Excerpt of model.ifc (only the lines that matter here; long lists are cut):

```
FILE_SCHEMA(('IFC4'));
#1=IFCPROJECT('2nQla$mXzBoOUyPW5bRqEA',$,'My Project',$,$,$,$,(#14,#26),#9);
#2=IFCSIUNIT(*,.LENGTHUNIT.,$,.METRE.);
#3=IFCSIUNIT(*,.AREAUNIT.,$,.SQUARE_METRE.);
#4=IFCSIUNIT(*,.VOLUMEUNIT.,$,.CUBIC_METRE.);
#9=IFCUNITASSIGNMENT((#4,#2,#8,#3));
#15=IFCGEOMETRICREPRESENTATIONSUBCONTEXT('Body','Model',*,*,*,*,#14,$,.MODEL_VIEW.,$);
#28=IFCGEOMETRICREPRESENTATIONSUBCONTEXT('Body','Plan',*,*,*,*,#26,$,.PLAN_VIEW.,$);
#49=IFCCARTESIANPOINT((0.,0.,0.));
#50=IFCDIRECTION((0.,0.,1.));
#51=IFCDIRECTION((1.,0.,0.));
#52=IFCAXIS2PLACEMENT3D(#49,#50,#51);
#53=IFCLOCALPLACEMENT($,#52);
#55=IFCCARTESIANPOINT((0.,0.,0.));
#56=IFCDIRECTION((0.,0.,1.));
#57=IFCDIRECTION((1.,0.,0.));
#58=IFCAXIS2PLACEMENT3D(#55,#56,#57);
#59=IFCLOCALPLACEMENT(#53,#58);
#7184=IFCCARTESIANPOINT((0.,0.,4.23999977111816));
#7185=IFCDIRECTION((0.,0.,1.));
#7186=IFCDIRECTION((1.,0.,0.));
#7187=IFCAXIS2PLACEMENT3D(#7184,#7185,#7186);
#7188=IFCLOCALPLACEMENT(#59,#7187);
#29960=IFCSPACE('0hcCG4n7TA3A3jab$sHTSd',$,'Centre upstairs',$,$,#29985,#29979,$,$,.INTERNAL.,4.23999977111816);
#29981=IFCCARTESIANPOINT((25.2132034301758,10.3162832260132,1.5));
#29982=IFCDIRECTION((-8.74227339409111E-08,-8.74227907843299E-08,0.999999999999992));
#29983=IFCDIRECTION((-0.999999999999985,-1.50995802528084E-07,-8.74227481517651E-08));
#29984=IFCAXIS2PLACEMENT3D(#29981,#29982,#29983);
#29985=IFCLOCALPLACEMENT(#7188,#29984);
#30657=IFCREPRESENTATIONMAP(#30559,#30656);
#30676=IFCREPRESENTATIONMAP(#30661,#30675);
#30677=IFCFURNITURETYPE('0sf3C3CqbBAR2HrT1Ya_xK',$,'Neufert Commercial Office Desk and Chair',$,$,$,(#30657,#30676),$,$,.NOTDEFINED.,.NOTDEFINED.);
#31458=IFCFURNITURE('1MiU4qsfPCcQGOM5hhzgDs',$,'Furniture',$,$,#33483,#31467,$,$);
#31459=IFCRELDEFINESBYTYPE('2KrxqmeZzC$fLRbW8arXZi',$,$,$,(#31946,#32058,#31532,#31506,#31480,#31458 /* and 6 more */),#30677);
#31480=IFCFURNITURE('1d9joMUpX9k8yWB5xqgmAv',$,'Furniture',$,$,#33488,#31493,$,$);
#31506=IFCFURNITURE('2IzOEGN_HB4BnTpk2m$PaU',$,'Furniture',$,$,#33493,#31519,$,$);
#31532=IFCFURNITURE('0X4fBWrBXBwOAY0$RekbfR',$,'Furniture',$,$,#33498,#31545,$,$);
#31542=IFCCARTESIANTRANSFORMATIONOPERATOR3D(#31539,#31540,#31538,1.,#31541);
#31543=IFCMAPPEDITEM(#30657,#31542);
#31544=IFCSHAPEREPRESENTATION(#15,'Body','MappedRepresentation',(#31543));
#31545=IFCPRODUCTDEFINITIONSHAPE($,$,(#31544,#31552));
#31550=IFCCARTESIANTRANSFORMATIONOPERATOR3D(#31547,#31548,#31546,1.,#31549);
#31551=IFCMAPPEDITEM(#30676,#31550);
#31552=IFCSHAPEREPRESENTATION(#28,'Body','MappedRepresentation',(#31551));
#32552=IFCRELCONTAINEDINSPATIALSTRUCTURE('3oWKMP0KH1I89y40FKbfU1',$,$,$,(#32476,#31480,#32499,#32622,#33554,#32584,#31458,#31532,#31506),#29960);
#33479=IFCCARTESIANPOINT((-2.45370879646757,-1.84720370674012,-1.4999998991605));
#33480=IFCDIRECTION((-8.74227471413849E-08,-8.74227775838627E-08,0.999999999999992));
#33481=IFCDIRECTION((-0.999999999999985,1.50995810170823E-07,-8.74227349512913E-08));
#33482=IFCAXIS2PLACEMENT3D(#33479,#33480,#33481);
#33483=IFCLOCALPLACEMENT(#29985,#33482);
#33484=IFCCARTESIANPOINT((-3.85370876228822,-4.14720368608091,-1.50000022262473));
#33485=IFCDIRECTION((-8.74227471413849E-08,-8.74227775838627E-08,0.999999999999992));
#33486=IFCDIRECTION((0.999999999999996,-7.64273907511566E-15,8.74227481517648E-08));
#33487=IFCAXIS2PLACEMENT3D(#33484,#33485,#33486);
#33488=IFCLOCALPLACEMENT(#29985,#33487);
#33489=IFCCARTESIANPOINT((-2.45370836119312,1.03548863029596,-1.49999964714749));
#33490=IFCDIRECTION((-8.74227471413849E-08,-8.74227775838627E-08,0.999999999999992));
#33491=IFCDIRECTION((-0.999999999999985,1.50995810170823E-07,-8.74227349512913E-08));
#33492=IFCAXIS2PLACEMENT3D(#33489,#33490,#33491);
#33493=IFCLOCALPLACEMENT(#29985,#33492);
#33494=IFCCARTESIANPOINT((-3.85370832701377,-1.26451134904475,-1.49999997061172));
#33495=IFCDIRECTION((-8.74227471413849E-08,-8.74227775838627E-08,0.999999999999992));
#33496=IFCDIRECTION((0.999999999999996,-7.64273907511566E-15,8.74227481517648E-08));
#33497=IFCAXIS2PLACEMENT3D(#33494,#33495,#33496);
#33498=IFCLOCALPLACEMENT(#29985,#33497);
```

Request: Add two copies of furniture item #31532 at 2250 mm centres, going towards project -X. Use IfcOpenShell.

```python
import numpy as np
import ifcopenshell
import ifcopenshell.api.geometry
import ifcopenshell.api.root
import ifcopenshell.util.element
import ifcopenshell.util.placement
import ifcopenshell.util.unit

model = ifcopenshell.open("model.ifc")
unit_scale = ifcopenshell.util.unit.calculate_unit_scale(model)

source = model.by_guid("0X4fBWrBXBwOAY0$RekbfR")
base = ifcopenshell.util.placement.get_local_placement(source.ObjectPlacement)
step = np.array([-1.0, 0.0, 0.0]) * 2.25 / unit_scale

for i in range(1, 3):
    copy = ifcopenshell.api.root.copy_class(model, product=source)
    copy.Representation = ifcopenshell.util.element.copy_deep(
        model, source.Representation, exclude=["IfcGeometricRepresentationContext", "IfcRepresentationMap"]
    )
    matrix = base.copy()
    matrix[:3, 3] += i * step
    print("added at", matrix[:3, 3].round(3) + 0.0)
    ifcopenshell.api.geometry.edit_object_placement(model, product=copy, matrix=matrix, is_si=False)

model.write("model_edited.ifc")
```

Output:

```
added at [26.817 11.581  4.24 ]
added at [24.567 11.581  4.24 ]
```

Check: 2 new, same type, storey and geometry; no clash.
